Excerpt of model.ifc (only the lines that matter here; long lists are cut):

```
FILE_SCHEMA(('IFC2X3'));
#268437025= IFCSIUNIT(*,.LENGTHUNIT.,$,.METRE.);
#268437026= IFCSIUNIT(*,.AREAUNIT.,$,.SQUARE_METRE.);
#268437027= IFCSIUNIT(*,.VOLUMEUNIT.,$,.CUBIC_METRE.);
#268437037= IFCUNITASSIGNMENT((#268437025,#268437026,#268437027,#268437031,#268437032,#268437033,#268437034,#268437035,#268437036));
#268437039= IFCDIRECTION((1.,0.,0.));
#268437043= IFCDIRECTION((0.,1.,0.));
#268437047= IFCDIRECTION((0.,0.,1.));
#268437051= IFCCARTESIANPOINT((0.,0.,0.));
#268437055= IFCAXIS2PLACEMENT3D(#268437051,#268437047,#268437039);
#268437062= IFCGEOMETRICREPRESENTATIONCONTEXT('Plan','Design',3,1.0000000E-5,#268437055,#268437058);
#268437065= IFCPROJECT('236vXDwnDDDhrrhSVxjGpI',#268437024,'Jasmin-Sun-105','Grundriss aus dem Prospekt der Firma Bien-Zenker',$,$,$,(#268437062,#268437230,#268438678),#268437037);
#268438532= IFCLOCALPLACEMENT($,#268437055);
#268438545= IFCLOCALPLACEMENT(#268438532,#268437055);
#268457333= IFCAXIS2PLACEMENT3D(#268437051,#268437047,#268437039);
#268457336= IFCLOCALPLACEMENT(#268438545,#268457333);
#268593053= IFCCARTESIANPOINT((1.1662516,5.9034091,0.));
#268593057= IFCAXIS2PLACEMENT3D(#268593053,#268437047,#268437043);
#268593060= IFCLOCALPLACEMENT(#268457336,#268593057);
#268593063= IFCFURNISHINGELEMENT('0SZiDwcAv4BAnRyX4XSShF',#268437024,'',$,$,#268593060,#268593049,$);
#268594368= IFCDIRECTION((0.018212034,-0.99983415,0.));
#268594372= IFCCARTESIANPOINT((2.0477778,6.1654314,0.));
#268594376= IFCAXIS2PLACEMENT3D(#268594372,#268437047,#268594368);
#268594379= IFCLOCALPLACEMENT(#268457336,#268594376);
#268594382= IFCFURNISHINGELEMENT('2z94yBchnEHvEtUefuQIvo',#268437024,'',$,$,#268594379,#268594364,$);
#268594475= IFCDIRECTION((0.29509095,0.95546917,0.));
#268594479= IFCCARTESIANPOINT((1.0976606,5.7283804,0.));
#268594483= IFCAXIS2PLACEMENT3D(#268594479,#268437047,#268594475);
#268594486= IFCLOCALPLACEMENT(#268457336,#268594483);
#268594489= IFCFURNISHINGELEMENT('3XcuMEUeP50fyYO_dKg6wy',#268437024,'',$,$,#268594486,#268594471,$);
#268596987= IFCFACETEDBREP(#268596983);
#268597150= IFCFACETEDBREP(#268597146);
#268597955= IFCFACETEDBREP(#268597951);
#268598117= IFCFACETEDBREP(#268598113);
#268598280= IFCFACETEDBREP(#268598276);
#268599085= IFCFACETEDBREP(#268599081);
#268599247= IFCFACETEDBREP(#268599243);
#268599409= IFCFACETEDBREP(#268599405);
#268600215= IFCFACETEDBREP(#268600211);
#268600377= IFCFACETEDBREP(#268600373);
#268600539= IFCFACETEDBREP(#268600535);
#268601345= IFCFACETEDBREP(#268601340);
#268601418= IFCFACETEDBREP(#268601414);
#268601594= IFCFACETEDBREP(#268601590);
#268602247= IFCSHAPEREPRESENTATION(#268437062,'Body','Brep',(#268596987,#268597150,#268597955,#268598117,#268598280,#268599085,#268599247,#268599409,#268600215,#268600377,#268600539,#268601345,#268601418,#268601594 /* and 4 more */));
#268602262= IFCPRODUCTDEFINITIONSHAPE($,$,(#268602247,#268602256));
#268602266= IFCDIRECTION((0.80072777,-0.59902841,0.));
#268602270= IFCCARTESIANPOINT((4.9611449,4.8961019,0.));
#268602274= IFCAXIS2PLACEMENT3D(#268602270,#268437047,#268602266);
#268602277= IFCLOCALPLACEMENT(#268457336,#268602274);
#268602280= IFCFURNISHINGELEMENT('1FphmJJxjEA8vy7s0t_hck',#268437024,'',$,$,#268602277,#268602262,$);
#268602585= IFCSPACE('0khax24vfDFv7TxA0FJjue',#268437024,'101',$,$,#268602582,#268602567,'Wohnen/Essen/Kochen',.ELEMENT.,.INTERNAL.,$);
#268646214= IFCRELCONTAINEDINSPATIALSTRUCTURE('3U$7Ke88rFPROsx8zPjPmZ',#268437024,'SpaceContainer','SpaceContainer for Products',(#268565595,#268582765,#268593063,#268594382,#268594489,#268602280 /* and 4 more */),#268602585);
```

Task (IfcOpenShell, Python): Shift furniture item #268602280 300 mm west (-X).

```python
import ifcopenshell
import ifcopenshell.api.geometry
import ifcopenshell.util.placement
import ifcopenshell.util.unit

model = ifcopenshell.open("model.ifc")
unit_scale = ifcopenshell.util.unit.calculate_unit_scale(model)

item = model.by_guid("1FphmJJxjEA8vy7s0t_hck")
matrix = ifcopenshell.util.placement.get_local_placement(item.ObjectPlacement)
matrix[0, 3] -= 0.3 / unit_scale
ifcopenshell.api.geometry.edit_object_placement(model, product=item, matrix=matrix, is_si=False)

print(ifcopenshell.util.placement.get_local_placement(item.ObjectPlacement).round(3) + 0.0)

model.write("model_edited.ifc")
```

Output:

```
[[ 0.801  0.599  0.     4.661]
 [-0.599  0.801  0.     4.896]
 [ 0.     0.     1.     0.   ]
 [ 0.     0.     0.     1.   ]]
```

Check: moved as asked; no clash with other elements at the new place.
